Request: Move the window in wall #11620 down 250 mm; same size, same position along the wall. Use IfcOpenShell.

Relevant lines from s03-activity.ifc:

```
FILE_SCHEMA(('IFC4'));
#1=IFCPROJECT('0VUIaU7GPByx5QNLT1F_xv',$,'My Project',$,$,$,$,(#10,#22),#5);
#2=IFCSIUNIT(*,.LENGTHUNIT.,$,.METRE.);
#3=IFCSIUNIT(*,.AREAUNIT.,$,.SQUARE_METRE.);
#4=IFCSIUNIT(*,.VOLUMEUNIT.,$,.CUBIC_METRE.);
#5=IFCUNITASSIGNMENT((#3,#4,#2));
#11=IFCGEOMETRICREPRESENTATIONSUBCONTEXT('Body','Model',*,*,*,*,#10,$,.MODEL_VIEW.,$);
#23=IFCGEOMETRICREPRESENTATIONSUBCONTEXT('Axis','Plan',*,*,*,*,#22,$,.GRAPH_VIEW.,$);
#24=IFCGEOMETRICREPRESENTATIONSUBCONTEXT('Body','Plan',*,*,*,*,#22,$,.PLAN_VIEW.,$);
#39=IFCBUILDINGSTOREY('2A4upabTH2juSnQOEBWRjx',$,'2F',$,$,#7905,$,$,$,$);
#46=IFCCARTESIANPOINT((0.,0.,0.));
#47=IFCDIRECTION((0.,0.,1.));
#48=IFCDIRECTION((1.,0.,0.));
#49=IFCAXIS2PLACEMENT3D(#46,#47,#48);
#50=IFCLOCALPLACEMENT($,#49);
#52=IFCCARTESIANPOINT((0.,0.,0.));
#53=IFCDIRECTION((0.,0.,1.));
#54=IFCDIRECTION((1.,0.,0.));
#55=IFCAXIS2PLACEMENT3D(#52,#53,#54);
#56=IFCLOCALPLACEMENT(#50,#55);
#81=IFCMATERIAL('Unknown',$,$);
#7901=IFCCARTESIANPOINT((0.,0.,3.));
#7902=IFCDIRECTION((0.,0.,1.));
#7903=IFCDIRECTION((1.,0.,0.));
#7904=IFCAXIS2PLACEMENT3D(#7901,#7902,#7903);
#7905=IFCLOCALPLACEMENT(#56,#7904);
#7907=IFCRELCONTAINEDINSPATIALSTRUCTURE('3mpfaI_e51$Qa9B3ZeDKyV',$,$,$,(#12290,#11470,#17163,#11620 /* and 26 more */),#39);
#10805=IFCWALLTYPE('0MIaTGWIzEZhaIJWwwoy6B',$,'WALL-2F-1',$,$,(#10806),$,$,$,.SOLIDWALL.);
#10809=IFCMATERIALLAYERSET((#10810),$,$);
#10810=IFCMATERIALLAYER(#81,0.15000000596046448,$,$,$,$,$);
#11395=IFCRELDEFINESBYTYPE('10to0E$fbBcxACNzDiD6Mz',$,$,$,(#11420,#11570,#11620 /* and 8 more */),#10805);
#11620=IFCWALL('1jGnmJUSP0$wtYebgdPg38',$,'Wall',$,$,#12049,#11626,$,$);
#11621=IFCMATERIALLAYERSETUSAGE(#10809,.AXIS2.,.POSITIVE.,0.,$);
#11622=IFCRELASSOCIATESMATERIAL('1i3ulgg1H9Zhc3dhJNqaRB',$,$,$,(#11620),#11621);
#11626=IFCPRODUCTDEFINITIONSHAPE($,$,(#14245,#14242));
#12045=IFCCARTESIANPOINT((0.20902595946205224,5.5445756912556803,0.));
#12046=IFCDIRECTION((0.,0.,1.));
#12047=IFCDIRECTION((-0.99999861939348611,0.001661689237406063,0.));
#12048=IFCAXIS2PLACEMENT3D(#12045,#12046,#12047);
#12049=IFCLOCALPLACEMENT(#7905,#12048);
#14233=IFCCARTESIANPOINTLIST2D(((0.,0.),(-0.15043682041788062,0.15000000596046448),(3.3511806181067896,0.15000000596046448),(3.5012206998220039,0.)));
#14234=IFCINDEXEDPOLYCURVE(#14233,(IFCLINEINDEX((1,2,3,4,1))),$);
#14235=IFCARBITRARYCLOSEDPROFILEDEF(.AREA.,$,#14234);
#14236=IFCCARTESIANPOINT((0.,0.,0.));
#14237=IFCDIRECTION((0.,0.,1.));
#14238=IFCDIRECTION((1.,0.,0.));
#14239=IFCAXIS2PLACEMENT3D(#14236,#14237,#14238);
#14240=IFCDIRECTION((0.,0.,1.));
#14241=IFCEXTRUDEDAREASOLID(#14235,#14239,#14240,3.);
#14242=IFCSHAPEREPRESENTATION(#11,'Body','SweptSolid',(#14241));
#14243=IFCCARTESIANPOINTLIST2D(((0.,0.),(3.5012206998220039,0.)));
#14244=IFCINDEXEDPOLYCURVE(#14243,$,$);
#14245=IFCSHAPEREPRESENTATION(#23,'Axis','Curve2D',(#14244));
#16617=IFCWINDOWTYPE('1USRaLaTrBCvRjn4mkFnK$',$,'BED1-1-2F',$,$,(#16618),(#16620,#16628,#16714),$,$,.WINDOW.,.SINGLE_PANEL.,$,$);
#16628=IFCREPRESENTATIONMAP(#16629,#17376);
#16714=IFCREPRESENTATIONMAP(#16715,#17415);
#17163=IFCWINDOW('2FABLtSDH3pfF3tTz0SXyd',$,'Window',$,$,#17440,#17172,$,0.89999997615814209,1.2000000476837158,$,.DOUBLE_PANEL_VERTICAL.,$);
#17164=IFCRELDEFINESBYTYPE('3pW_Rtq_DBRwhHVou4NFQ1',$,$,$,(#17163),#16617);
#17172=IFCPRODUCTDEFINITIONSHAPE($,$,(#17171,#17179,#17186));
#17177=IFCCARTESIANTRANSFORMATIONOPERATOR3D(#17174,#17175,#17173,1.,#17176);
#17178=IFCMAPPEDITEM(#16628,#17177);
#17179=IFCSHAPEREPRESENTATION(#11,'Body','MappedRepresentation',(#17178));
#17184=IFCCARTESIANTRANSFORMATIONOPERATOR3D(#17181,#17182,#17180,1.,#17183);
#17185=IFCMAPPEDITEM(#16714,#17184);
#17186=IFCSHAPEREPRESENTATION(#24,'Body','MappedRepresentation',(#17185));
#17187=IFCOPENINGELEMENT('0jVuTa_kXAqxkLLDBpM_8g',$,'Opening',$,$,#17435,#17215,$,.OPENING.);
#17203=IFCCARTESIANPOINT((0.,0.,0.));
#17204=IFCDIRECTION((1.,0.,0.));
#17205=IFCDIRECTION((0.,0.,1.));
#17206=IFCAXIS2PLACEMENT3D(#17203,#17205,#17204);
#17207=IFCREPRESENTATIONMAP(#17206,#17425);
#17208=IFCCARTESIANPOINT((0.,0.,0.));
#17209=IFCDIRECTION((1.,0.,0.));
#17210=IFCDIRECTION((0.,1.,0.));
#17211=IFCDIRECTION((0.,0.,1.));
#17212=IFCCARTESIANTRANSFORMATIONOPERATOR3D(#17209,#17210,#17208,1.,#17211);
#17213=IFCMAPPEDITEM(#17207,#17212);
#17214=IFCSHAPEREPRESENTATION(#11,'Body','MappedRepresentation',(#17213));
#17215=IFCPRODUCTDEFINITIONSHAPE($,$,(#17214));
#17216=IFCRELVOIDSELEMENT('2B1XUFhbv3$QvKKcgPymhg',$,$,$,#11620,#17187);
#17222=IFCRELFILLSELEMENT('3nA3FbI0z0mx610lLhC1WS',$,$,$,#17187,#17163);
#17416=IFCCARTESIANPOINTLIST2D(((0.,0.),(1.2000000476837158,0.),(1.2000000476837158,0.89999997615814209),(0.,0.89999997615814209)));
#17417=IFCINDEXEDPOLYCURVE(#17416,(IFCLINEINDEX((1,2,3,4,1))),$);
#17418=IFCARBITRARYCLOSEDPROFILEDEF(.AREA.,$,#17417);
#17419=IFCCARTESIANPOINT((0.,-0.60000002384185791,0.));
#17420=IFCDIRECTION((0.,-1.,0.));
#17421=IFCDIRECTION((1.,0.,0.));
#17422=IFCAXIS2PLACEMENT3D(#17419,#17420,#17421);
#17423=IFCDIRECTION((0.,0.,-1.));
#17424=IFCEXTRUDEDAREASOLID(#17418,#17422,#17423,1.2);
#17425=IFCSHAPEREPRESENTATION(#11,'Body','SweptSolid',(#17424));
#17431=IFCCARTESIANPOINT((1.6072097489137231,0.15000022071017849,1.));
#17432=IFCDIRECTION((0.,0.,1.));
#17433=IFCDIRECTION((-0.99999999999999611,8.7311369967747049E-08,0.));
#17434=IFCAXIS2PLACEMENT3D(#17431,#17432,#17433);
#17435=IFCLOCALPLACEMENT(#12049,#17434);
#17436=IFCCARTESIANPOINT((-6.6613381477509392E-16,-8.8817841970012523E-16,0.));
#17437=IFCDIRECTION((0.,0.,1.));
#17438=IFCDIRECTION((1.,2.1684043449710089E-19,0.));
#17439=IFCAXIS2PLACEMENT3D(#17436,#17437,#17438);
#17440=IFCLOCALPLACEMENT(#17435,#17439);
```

```python
import numpy as np
import ifcopenshell
import ifcopenshell.api.geometry
import ifcopenshell.util.placement
import ifcopenshell.util.unit

model = ifcopenshell.open("s03-activity.ifc")
unit_scale = ifcopenshell.util.unit.calculate_unit_scale(model)

window = model.by_guid("2FABLtSDH3pfF3tTz0SXyd")
opening = window.FillsVoids[0].RelatingOpeningElement
dz = -0.25 / unit_scale

shift = np.array([0.0, 0.0, dz])
# The window is placed relative to its opening, so it follows when the opening moves.
matrix = ifcopenshell.util.placement.get_local_placement(opening.ObjectPlacement)
matrix[:3, 3] += shift
ifcopenshell.api.geometry.edit_object_placement(
    model, product=opening, matrix=matrix, is_si=False, should_transform_children=True
)

print(f"moved by {dz * unit_scale:+.3f} m")

model.write("s03-activity_rev.ifc")
```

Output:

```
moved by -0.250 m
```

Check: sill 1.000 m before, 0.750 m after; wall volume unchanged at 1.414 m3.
